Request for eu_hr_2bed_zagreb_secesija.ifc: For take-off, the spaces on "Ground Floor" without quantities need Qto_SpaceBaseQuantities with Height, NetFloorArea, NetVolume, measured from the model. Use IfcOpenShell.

First a look at what the model holds.

```python
import ifcopenshell
import ifcopenshell.util.element
import ifcopenshell.util.unit

model = ifcopenshell.open("eu_hr_2bed_zagreb_secesija.ifc")
print(model.schema)
for unit_type in ("LENGTHUNIT", "AREAUNIT", "VOLUMEUNIT"):
    print(unit_type, ifcopenshell.util.unit.calculate_unit_scale(model, unit_type))
storey = next(s for s in model.by_type("IfcBuildingStorey") if s.Name == "Ground Floor")
spaces = [e for e in ifcopenshell.util.element.get_decomposition(storey) if e.is_a("IfcSpace")]
for e in sorted(spaces, key=lambda e: e.id()):
    print(e.id(), e.is_a(), e.Name, list(ifcopenshell.util.element.get_psets(e, qtos_only=True)), sep=" | ")
```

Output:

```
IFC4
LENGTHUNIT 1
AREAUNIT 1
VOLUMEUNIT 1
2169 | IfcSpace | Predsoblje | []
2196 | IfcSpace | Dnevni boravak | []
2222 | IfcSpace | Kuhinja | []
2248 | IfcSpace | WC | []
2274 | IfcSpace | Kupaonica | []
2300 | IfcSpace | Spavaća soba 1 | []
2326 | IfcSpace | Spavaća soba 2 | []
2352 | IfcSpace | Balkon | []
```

```python
import ifcopenshell
import ifcopenshell.api.pset
import ifcopenshell.geom
import ifcopenshell.util.element
import ifcopenshell.util.shape
import ifcopenshell.util.unit

model = ifcopenshell.open("eu_hr_2bed_zagreb_secesija.ifc")
unit_scale = ifcopenshell.util.unit.calculate_unit_scale(model)
area_scale = ifcopenshell.util.unit.calculate_unit_scale(model, "AREAUNIT")
volume_scale = ifcopenshell.util.unit.calculate_unit_scale(model, "VOLUMEUNIT")
settings = ifcopenshell.geom.settings()

storey = next(s for s in model.by_type("IfcBuildingStorey") if s.Name == "Ground Floor")
spaces = [e for e in ifcopenshell.util.element.get_decomposition(storey) if e.is_a("IfcSpace")]

for e in sorted(spaces, key=lambda e: e.id()):
    if ifcopenshell.util.element.get_psets(e, qtos_only=True, should_inherit=False):
        continue
    # Geometry comes back in metres, in the element's own axes.
    shape = ifcopenshell.geom.create_shape(settings, e)
    values = {
        "Height": ifcopenshell.util.shape.get_z(shape.geometry) / unit_scale,
        "NetFloorArea": ifcopenshell.util.shape.get_footprint_area(shape.geometry) / area_scale,
        "NetVolume": ifcopenshell.util.shape.get_volume(shape.geometry) / volume_scale,
    }
    qto = ifcopenshell.api.pset.add_qto(model, product=e, name="Qto_SpaceBaseQuantities")
    ifcopenshell.api.pset.edit_qto(model, qto=qto, properties=values)
    print(e.id(), {k: round(v, 3) for k, v in values.items()})

model.write("eu_hr_2bed_zagreb_secesija_edited.ifc")
```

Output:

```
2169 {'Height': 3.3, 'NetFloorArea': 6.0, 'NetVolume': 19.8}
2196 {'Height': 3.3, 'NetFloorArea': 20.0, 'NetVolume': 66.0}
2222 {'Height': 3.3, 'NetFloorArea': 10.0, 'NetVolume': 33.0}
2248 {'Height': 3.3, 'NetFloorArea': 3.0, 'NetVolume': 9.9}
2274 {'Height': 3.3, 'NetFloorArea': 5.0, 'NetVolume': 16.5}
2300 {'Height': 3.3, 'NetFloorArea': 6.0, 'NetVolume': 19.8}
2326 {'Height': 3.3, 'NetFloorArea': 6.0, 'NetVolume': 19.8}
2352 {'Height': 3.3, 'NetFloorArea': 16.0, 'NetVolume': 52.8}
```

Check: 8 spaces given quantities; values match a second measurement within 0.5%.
